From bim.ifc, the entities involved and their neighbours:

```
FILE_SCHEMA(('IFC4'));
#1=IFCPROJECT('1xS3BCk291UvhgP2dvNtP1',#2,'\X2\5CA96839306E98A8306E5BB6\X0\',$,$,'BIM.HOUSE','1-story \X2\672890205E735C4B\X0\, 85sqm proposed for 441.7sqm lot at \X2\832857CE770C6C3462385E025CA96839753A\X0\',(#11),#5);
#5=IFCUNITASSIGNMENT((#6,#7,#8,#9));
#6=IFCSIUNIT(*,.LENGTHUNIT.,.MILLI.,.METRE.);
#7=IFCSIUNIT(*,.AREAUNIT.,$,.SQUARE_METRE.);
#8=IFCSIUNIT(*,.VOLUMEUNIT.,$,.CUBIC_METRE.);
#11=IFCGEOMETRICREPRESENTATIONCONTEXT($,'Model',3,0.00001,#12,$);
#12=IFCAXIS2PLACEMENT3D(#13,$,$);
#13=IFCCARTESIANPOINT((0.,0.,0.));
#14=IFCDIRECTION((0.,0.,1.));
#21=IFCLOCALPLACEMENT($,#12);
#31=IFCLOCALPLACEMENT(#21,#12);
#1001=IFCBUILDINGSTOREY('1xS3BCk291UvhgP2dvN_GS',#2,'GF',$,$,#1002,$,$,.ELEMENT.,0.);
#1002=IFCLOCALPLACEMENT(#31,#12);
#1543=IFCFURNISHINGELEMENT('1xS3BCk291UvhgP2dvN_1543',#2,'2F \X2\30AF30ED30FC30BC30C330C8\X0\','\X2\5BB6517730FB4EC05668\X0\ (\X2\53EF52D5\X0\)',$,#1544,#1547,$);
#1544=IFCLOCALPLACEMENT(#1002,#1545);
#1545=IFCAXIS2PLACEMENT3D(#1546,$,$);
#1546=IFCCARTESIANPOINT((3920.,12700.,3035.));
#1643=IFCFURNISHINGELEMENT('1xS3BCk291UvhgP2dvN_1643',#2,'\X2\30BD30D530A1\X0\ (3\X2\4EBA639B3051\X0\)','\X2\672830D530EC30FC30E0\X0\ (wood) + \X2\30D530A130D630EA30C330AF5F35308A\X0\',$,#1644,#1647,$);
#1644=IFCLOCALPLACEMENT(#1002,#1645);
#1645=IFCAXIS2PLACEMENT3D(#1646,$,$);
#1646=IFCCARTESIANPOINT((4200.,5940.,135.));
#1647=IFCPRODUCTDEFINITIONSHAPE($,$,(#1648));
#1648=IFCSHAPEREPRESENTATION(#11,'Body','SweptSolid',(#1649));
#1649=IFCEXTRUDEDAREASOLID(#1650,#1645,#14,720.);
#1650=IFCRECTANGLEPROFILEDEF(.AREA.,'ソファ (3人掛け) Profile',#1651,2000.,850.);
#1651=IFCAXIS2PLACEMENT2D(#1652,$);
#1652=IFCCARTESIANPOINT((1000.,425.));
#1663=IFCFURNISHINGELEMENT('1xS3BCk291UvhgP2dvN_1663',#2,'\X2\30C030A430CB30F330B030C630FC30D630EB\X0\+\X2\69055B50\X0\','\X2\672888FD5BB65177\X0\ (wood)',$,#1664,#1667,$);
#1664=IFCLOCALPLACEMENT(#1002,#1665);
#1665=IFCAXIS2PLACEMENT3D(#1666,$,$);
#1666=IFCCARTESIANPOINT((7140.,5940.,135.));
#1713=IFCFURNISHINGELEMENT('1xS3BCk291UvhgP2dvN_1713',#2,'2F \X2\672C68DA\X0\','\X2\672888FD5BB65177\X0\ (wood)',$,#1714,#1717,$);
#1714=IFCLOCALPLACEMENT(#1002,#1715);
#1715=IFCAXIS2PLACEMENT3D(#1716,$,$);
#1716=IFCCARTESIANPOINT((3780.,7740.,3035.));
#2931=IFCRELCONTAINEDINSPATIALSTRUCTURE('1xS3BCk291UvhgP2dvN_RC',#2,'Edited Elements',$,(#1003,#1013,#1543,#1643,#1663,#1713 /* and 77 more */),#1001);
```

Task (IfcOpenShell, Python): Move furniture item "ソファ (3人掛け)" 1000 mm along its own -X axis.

```python
import ifcopenshell
import ifcopenshell.api.geometry
import ifcopenshell.util.placement
import ifcopenshell.util.unit

model = ifcopenshell.open("bim.ifc")
unit_scale = ifcopenshell.util.unit.calculate_unit_scale(model)

item = model.by_guid("1xS3BCk291UvhgP2dvN_1643")
matrix = ifcopenshell.util.placement.get_local_placement(item.ObjectPlacement)
matrix[:3, 3] -= matrix[:3, 0] * 1 / unit_scale
ifcopenshell.api.geometry.edit_object_placement(model, product=item, matrix=matrix, is_si=False)

print(ifcopenshell.util.placement.get_local_placement(item.ObjectPlacement).round(3) + 0.0)

model.write("bim-out.ifc")
```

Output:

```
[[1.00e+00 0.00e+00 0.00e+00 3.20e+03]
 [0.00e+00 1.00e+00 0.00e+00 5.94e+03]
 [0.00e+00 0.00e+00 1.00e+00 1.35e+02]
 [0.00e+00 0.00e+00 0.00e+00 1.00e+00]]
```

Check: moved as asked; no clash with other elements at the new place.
